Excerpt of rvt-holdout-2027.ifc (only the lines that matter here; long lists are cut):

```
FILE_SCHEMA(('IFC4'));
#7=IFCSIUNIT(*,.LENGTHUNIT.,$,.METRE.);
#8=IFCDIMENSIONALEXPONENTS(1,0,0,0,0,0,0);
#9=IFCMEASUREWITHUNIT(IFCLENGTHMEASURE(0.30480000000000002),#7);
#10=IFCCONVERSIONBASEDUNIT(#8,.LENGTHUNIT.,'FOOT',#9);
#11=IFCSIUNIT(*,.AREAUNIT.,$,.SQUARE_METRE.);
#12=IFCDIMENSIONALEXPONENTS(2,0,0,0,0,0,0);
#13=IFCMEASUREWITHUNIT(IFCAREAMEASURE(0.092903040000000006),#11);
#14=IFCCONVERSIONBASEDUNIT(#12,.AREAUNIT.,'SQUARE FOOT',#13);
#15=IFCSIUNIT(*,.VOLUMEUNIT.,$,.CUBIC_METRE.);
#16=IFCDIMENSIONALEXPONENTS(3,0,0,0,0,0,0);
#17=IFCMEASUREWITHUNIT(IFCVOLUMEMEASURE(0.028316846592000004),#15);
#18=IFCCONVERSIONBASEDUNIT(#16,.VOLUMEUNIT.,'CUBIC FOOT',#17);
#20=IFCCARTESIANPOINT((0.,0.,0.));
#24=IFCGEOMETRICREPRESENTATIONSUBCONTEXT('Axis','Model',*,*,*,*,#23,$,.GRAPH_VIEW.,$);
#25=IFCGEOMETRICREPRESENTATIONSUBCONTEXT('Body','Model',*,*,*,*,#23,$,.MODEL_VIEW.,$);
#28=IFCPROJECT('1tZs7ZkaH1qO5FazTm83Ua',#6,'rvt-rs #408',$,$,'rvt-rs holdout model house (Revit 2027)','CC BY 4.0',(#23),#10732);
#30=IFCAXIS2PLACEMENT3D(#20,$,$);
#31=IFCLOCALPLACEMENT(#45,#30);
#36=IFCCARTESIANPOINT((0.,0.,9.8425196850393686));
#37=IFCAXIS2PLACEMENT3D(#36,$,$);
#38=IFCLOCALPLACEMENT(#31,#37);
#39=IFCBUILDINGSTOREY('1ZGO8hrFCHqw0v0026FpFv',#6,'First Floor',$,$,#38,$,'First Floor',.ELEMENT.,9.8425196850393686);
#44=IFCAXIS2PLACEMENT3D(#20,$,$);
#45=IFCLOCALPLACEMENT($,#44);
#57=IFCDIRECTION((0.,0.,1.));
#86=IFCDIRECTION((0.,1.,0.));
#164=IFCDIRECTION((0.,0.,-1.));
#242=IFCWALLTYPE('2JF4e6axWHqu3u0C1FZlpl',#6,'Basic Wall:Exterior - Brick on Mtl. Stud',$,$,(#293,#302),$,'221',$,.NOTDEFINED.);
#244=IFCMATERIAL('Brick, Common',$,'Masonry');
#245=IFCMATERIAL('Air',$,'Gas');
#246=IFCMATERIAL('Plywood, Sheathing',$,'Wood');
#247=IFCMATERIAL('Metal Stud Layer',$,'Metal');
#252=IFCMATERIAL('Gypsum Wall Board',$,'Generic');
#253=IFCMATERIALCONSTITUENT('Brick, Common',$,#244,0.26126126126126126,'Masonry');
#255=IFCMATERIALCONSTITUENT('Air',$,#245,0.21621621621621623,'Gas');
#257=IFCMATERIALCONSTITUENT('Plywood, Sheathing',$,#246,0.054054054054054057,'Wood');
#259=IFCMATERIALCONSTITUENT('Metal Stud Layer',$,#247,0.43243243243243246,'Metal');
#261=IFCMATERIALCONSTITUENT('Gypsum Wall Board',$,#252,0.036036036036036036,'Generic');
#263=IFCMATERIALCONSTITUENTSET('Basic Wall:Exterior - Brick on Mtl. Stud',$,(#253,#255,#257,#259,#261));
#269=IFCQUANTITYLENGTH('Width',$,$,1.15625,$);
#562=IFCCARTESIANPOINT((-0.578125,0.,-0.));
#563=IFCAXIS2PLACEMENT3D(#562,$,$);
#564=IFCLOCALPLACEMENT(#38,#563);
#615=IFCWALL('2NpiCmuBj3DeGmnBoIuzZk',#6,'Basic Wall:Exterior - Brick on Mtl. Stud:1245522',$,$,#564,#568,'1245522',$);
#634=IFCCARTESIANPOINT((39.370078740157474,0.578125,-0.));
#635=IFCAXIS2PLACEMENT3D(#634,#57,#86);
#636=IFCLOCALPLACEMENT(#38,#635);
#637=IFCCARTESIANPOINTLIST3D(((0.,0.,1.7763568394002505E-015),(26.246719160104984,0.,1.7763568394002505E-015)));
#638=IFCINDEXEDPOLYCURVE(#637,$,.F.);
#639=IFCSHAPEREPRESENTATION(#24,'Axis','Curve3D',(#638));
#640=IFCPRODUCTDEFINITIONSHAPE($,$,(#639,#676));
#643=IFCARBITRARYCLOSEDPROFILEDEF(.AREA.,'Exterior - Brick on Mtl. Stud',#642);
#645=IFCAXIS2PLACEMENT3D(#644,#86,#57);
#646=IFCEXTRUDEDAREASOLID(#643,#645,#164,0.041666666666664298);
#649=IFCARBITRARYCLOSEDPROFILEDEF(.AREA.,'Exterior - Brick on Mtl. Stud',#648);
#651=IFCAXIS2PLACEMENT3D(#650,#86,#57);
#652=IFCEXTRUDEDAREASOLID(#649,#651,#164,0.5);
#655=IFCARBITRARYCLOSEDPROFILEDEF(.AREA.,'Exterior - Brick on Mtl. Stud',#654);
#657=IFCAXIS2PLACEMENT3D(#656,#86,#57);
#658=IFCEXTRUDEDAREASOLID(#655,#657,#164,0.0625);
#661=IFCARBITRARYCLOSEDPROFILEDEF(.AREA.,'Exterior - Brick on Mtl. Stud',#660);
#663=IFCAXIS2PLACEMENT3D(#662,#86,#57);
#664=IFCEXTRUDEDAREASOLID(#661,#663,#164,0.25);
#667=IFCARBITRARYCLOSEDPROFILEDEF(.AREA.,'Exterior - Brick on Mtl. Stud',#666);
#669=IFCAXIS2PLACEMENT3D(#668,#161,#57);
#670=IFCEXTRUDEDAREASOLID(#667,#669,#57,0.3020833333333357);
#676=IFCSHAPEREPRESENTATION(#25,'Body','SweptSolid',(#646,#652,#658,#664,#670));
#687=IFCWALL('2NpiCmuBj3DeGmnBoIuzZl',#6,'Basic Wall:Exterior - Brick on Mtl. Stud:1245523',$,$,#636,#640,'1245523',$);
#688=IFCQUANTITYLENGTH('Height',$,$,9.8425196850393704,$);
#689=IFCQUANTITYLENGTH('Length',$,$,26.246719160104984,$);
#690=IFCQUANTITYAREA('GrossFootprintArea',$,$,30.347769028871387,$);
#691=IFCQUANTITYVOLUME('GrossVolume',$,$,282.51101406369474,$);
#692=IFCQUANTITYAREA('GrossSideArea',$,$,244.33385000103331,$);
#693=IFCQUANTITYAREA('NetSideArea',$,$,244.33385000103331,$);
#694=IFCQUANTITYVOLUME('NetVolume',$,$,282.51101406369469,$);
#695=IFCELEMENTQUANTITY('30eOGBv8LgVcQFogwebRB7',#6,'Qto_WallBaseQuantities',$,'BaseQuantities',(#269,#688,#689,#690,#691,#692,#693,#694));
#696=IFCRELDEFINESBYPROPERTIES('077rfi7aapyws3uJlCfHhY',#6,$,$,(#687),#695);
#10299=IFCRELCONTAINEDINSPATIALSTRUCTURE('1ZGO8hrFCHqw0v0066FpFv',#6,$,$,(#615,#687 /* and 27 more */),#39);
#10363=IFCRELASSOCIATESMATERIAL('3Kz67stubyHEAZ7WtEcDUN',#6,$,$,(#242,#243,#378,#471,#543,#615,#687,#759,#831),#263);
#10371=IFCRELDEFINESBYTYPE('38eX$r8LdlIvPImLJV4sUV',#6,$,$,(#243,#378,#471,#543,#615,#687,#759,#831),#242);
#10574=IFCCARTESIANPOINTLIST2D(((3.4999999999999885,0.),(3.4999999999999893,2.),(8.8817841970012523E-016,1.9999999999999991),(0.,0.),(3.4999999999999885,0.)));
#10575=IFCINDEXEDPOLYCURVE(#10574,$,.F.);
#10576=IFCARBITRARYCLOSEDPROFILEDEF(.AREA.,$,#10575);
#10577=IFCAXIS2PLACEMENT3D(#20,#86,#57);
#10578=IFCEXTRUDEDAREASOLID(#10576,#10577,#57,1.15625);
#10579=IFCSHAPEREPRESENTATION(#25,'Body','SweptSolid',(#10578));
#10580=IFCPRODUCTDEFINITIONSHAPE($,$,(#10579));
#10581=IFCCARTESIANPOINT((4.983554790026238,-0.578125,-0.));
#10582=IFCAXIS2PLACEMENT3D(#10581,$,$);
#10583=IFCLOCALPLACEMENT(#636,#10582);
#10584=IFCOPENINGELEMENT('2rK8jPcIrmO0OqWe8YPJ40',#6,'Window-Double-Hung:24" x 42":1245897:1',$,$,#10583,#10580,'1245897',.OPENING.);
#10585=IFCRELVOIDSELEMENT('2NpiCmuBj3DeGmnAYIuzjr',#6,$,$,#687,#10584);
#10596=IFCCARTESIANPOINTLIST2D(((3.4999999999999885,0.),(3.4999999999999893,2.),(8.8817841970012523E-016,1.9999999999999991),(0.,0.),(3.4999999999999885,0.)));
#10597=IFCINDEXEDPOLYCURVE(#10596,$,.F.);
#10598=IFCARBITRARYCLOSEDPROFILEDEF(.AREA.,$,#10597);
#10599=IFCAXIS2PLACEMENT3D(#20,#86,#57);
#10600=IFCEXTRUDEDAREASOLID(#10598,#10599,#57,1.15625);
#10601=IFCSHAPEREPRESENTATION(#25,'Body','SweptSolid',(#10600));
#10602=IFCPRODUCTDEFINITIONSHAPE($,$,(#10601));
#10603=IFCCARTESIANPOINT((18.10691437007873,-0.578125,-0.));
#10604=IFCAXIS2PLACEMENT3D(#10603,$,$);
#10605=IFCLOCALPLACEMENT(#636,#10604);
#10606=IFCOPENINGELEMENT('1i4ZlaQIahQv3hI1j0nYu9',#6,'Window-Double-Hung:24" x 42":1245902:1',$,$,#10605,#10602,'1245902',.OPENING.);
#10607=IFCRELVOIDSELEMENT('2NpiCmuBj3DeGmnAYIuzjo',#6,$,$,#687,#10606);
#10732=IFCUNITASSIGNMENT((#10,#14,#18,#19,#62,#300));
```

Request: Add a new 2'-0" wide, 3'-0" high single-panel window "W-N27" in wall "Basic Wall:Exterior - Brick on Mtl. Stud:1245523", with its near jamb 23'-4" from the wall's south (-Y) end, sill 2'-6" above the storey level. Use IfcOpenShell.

```python
import numpy as np
import ifcopenshell
import ifcopenshell.api.feature
import ifcopenshell.api.geometry
import ifcopenshell.api.pset
import ifcopenshell.api.root
import ifcopenshell.api.spatial
import ifcopenshell.geom
import ifcopenshell.util.element
import ifcopenshell.util.placement
import ifcopenshell.util.representation
import ifcopenshell.util.shape
import ifcopenshell.util.unit

model = ifcopenshell.open("rvt-holdout-2027.ifc")
unit_scale = ifcopenshell.util.unit.calculate_unit_scale(model)
area_scale = ifcopenshell.util.unit.calculate_unit_scale(model, "AREAUNIT")
volume_scale = ifcopenshell.util.unit.calculate_unit_scale(model, "VOLUMEUNIT")
settings = ifcopenshell.geom.settings()


def volume(element):
    """Net volume in cubic metres, openings subtracted."""
    shape = ifcopenshell.geom.create_shape(settings, element)
    return ifcopenshell.util.shape.get_volume(shape.geometry)


wall = model.by_id(687)
storey = ifcopenshell.util.element.get_container(wall, ifc_class="IfcBuildingStorey")
context = ifcopenshell.util.representation.get_context(model, "Model", "Body", "MODEL_VIEW")
before = volume(wall)

width, height, from_end, sill = 0.6096, 0.9144, 7.112, 0.762  # metres

# The wall runs along its own X axis, and the end named is its -X end.
wall_shape = ifcopenshell.geom.create_shape(settings, wall)
x, y, z = ifcopenshell.util.shape.get_vertices(wall_shape.geometry).T
start = x.min() + from_end
face, thickness = float(y.min()), float(y.max() - y.min())
wall_matrix = ifcopenshell.util.placement.get_local_placement(wall.ObjectPlacement)
level = ifcopenshell.util.placement.get_local_placement(storey.ObjectPlacement)[2, 3]


def in_wall(x, y):
    """Placement at x, y metres in the wall's axes, at sill height."""
    matrix = wall_matrix.copy()
    matrix[:, 3] = wall_matrix @ np.array([x / unit_scale, y / unit_scale, 0.0, 1.0])
    matrix[2, 3] = level + sill / unit_scale
    return matrix


# Opening: a box that overshoots both wall faces by 50 mm.
opening = ifcopenshell.api.root.create_entity(model, ifc_class="IfcOpeningElement", predefined_type="OPENING")
box = ifcopenshell.api.geometry.add_wall_representation(
    model, context=context, length=width, height=height, thickness=thickness + 0.1
)
ifcopenshell.api.geometry.assign_representation(model, product=opening, representation=box)
ifcopenshell.api.geometry.edit_object_placement(model, product=opening, matrix=in_wall(start, face - 0.05), is_si=False)
ifcopenshell.api.feature.add_feature(model, feature=opening, element=wall)

window = ifcopenshell.api.root.create_entity(model, ifc_class="IfcWindow", name="W-N27", predefined_type="WINDOW")
window.OverallWidth, window.OverallHeight = width / unit_scale, height / unit_scale
window.PartitioningType = "SINGLE_PANEL"
body = ifcopenshell.api.geometry.add_window_representation(
    model,
    context=context,
    overall_width=window.OverallWidth,
    overall_height=window.OverallHeight,
    partition_type="SINGLE_PANEL",
)
ifcopenshell.api.geometry.assign_representation(model, product=window, representation=body)
ifcopenshell.api.spatial.assign_container(model, products=[window], relating_structure=storey)
ifcopenshell.api.feature.add_filling(model, opening=opening, element=window)

# Centre the window in the wall's thickness.
ifcopenshell.api.geometry.edit_object_placement(model, product=window, matrix=in_wall(start, face), is_si=False)
window_shape = ifcopenshell.geom.create_shape(settings, window)
depth = ifcopenshell.util.shape.get_vertices(window_shape.geometry)[:, 1]
offset = face + thickness / 2 - (depth.min() + depth.max()) / 2
ifcopenshell.api.geometry.edit_object_placement(model, product=window, matrix=in_wall(start, offset), is_si=False)

after = volume(wall)

# Update the wall's stored quantities.
qto = model.by_id(ifcopenshell.util.element.get_pset(wall, "Qto_WallBaseQuantities", should_inherit=False)["id"])
ifcopenshell.api.pset.edit_qto(model, qto=qto, properties={
    "NetSideArea": after / thickness / area_scale,
    "NetVolume": after / volume_scale,
})

print(f"wall volume {before:.3f} -> {after:.3f} m3")

model.write("rvt-holdout-2027_rev.ifc")
```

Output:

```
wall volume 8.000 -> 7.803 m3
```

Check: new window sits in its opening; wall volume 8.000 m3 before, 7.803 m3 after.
